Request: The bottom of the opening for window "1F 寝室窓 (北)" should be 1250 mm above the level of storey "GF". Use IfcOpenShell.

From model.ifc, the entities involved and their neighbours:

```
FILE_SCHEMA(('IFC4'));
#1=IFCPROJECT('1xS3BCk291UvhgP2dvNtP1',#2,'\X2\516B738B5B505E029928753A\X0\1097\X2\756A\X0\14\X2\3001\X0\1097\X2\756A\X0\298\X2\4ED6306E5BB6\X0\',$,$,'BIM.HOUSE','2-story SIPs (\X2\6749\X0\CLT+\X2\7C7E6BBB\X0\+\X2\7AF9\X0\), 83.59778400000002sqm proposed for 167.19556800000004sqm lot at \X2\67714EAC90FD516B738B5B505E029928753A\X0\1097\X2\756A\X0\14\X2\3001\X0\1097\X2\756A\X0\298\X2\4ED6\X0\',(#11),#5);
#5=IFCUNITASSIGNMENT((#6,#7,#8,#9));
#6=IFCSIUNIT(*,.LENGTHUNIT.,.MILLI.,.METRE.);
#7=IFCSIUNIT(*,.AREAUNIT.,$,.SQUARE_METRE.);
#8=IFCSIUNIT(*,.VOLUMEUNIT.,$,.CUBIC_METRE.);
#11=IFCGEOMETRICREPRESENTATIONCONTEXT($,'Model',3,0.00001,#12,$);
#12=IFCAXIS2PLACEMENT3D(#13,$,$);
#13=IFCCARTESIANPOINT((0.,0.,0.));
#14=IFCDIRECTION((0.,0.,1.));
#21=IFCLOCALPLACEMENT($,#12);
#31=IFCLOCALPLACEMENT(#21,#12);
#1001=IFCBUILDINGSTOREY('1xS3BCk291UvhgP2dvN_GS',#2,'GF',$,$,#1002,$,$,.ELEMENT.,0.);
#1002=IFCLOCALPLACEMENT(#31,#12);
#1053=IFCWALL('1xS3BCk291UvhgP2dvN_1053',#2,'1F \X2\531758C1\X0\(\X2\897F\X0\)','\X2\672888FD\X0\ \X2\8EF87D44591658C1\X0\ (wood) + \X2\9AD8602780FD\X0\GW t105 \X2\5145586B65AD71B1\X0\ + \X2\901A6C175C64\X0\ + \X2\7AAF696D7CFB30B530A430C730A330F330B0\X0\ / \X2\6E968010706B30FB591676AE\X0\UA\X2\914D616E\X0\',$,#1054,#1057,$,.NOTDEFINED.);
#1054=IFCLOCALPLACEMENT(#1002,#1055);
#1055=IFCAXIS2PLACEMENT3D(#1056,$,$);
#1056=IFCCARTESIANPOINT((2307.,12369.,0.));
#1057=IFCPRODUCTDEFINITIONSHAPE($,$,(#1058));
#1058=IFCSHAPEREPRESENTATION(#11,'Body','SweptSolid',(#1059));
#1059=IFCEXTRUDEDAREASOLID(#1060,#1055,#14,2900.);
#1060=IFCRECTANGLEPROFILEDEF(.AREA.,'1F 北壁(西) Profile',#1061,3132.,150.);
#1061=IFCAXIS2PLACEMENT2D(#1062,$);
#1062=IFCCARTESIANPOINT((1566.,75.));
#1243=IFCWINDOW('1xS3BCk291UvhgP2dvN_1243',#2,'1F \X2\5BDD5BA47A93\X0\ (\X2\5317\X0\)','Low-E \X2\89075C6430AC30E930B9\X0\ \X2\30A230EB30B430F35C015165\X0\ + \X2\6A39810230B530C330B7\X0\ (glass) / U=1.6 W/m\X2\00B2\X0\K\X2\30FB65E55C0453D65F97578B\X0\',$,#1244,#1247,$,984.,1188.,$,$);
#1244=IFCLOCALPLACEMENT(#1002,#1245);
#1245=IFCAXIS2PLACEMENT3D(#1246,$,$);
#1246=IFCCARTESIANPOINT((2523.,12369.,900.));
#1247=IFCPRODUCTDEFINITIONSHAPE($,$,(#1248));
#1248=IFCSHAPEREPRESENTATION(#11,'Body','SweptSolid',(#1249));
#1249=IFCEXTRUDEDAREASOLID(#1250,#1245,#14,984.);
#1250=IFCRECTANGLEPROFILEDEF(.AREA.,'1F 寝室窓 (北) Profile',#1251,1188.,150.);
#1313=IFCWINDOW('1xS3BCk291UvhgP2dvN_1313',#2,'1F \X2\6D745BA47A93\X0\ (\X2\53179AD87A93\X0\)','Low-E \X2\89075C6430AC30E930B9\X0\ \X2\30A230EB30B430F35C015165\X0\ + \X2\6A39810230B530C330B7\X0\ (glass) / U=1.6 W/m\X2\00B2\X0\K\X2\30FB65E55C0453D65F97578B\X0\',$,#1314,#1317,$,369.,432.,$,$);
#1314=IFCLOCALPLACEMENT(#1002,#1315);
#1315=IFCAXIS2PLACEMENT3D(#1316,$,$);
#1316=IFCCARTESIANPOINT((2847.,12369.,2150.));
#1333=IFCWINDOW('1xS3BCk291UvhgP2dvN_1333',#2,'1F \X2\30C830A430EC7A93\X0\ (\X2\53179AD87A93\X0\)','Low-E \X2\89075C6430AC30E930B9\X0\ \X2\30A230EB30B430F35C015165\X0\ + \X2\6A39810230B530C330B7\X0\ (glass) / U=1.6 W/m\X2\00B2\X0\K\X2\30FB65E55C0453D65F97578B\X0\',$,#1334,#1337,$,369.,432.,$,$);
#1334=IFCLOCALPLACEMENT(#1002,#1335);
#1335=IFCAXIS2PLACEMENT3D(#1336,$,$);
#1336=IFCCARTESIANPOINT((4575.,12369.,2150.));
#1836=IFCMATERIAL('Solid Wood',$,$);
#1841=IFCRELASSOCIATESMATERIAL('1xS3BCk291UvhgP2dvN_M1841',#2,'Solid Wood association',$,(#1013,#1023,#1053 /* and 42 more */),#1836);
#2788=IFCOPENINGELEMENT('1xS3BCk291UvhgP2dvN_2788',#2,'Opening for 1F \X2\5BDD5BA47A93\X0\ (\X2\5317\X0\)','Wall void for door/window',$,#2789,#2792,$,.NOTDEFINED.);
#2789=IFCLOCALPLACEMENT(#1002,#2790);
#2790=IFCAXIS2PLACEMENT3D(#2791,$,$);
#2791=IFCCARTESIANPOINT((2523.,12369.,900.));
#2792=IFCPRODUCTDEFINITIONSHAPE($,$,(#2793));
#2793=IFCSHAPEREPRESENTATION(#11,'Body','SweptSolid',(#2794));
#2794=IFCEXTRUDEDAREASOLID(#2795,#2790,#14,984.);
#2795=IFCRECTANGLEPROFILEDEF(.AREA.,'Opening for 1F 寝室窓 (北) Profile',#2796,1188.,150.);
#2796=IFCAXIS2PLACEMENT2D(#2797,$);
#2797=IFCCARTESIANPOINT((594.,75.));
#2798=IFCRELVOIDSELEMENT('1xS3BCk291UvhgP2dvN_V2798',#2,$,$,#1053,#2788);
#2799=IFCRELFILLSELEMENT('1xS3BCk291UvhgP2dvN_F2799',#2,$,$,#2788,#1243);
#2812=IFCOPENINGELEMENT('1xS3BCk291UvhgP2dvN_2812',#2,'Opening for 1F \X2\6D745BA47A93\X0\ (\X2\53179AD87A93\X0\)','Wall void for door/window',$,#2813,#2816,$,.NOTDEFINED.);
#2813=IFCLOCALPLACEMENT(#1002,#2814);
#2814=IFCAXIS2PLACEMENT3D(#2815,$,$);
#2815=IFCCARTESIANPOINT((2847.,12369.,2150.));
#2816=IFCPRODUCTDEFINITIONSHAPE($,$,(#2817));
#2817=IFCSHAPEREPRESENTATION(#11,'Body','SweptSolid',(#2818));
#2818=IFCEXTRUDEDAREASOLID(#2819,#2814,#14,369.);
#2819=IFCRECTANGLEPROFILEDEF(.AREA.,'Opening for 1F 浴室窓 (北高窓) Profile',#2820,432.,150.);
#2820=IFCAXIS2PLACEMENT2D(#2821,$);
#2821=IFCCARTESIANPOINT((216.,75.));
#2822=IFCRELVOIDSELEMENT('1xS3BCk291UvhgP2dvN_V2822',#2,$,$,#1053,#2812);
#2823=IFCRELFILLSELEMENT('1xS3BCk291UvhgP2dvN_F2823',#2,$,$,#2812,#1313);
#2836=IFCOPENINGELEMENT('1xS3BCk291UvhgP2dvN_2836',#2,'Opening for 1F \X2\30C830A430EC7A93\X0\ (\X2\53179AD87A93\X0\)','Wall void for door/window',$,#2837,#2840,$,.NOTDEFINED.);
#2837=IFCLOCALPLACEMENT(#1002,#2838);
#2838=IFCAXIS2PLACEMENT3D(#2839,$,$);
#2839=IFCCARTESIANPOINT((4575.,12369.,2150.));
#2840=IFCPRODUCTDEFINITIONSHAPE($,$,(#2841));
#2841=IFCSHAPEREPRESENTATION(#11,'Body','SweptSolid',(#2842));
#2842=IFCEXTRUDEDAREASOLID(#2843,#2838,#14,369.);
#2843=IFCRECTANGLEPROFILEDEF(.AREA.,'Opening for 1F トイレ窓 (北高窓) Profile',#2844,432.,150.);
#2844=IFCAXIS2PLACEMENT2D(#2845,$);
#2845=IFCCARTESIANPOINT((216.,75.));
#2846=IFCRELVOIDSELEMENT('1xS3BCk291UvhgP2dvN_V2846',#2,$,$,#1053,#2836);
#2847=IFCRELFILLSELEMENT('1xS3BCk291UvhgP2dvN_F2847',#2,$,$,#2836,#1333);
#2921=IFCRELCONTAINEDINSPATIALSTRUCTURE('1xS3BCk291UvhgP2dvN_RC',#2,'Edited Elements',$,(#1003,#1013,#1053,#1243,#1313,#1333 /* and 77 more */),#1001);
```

```python
import numpy as np
import ifcopenshell
import ifcopenshell.api.geometry
import ifcopenshell.geom
import ifcopenshell.util.element
import ifcopenshell.util.placement
import ifcopenshell.util.shape
import ifcopenshell.util.unit

model = ifcopenshell.open("model.ifc")
unit_scale = ifcopenshell.util.unit.calculate_unit_scale(model)

window = model.by_id(1243)
opening = window.FillsVoids[0].RelatingOpeningElement
storey = ifcopenshell.util.element.get_container(window, ifc_class="IfcBuildingStorey")
level = ifcopenshell.util.placement.get_local_placement(storey.ObjectPlacement)[2, 3]

# The opening's origin need not be at the sill, so measure its lowest point.
shape = ifcopenshell.geom.create_shape(ifcopenshell.geom.settings(), opening)
bottom = ifcopenshell.util.shape.get_shape_bottom_elevation(shape, shape.geometry) / unit_scale
dz = level + 1.25 / unit_scale - bottom

shift = np.array([0.0, 0.0, dz])
# The window is not placed relative to its opening, so move both.
for product in (opening, window):
    matrix = ifcopenshell.util.placement.get_local_placement(product.ObjectPlacement)
    matrix[:3, 3] += shift
    ifcopenshell.api.geometry.edit_object_placement(model, product=product, matrix=matrix, is_si=False)

print(f"moved by {dz * unit_scale:+.3f} m")

model.write("model_rev.ifc")
```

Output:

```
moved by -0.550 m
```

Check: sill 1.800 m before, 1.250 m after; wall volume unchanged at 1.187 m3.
